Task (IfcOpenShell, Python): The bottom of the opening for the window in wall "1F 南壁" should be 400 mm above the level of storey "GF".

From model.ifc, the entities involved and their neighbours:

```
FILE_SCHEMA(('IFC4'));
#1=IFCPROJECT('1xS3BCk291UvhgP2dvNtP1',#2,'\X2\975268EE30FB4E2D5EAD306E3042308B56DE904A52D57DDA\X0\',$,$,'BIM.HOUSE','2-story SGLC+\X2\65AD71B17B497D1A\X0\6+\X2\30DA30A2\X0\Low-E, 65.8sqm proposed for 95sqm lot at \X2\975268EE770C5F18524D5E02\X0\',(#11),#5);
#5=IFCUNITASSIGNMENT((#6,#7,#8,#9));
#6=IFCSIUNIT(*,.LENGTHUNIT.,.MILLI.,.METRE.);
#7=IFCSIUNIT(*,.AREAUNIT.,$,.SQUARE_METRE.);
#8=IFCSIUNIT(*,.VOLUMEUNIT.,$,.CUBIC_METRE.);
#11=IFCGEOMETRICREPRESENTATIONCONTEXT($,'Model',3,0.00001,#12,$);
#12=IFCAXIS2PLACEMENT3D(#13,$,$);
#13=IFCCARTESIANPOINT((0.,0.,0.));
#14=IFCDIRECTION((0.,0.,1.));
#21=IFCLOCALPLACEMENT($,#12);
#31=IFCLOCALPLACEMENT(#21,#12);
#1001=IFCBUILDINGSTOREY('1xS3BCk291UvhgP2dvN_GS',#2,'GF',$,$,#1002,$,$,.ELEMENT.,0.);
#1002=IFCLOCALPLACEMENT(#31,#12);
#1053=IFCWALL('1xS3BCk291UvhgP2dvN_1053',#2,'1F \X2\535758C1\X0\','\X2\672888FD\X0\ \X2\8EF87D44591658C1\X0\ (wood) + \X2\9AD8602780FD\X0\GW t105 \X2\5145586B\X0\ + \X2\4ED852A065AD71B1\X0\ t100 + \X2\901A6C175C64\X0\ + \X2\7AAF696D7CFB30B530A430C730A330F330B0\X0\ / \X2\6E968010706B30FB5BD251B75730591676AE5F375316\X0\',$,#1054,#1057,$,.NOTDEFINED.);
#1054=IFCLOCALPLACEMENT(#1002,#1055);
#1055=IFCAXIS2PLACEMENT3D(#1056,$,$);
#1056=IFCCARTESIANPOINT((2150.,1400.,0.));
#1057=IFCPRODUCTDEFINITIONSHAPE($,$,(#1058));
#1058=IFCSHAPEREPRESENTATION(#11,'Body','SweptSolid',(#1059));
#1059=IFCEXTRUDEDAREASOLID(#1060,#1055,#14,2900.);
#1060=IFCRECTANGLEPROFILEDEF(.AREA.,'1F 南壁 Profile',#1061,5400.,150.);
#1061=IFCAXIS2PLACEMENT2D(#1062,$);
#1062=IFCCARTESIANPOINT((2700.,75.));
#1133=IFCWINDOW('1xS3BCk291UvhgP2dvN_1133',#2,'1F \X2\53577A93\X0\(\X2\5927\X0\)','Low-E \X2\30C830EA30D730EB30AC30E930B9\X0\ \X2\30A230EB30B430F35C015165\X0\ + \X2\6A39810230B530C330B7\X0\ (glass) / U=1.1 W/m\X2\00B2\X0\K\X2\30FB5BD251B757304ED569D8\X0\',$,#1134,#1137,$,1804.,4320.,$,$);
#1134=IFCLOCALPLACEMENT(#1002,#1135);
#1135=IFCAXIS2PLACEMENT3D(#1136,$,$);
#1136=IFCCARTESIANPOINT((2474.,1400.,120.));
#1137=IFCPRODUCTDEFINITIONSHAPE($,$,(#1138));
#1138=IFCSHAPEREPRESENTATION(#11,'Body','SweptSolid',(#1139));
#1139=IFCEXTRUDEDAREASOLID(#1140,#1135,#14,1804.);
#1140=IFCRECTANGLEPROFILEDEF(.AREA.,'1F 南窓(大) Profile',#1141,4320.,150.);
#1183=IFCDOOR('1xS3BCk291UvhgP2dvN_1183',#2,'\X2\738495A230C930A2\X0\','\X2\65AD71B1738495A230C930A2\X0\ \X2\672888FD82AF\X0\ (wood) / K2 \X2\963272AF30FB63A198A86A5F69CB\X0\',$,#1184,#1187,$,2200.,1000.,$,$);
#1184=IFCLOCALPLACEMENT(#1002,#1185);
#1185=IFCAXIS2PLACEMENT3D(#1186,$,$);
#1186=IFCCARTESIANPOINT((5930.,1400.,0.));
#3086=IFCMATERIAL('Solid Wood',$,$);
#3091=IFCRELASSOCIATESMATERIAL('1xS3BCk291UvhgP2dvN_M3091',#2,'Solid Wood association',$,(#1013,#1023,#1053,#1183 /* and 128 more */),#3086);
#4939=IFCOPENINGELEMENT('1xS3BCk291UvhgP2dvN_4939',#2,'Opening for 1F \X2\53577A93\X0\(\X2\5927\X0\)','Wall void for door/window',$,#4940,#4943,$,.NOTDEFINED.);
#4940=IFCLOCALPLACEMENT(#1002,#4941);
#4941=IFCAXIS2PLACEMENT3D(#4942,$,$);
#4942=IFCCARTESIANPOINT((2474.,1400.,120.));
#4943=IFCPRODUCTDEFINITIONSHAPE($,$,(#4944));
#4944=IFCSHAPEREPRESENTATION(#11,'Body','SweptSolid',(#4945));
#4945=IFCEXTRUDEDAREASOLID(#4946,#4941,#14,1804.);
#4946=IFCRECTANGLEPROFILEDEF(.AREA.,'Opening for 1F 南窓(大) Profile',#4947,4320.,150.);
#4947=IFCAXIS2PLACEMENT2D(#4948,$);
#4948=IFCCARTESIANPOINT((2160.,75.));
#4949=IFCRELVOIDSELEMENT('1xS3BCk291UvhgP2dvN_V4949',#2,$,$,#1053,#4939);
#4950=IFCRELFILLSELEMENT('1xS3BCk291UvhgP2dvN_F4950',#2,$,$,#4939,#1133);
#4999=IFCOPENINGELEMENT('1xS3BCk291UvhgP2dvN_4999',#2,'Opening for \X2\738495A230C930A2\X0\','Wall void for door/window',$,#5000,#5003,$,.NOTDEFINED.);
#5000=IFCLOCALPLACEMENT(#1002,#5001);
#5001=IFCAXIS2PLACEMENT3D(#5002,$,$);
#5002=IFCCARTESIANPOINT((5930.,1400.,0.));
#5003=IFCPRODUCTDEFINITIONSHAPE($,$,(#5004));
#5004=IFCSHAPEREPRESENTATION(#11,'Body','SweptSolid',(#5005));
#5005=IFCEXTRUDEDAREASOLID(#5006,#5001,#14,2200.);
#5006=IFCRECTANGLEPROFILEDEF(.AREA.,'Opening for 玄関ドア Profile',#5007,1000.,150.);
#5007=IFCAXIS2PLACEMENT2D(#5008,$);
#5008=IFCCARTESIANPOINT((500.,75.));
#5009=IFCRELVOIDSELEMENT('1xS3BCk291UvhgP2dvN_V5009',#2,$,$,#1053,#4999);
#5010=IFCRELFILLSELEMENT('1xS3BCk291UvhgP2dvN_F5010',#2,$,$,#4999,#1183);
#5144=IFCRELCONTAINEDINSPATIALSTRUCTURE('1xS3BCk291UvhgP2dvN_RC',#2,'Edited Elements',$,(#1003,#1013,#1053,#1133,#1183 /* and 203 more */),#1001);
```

```python
import numpy as np
import ifcopenshell
import ifcopenshell.api.geometry
import ifcopenshell.geom
import ifcopenshell.util.element
import ifcopenshell.util.placement
import ifcopenshell.util.shape
import ifcopenshell.util.unit

model = ifcopenshell.open("model.ifc")
unit_scale = ifcopenshell.util.unit.calculate_unit_scale(model)

window = model.by_guid("1xS3BCk291UvhgP2dvN_1133")
opening = window.FillsVoids[0].RelatingOpeningElement
storey = ifcopenshell.util.element.get_container(window, ifc_class="IfcBuildingStorey")
level = ifcopenshell.util.placement.get_local_placement(storey.ObjectPlacement)[2, 3]

# The opening's origin need not be at the sill, so measure its lowest point.
shape = ifcopenshell.geom.create_shape(ifcopenshell.geom.settings(), opening)
bottom = ifcopenshell.util.shape.get_shape_bottom_elevation(shape, shape.geometry) / unit_scale
dz = level + 0.4 / unit_scale - bottom

shift = np.array([0.0, 0.0, dz])
# The window is not placed relative to its opening, so move both.
for product in (opening, window):
    matrix = ifcopenshell.util.placement.get_local_placement(product.ObjectPlacement)
    matrix[:3, 3] += shift
    ifcopenshell.api.geometry.edit_object_placement(model, product=product, matrix=matrix, is_si=False)

print(f"moved by {dz * unit_scale:+.3f} m")

model.write("model_updated.ifc")
```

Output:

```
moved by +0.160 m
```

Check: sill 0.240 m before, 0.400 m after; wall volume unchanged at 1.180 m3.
